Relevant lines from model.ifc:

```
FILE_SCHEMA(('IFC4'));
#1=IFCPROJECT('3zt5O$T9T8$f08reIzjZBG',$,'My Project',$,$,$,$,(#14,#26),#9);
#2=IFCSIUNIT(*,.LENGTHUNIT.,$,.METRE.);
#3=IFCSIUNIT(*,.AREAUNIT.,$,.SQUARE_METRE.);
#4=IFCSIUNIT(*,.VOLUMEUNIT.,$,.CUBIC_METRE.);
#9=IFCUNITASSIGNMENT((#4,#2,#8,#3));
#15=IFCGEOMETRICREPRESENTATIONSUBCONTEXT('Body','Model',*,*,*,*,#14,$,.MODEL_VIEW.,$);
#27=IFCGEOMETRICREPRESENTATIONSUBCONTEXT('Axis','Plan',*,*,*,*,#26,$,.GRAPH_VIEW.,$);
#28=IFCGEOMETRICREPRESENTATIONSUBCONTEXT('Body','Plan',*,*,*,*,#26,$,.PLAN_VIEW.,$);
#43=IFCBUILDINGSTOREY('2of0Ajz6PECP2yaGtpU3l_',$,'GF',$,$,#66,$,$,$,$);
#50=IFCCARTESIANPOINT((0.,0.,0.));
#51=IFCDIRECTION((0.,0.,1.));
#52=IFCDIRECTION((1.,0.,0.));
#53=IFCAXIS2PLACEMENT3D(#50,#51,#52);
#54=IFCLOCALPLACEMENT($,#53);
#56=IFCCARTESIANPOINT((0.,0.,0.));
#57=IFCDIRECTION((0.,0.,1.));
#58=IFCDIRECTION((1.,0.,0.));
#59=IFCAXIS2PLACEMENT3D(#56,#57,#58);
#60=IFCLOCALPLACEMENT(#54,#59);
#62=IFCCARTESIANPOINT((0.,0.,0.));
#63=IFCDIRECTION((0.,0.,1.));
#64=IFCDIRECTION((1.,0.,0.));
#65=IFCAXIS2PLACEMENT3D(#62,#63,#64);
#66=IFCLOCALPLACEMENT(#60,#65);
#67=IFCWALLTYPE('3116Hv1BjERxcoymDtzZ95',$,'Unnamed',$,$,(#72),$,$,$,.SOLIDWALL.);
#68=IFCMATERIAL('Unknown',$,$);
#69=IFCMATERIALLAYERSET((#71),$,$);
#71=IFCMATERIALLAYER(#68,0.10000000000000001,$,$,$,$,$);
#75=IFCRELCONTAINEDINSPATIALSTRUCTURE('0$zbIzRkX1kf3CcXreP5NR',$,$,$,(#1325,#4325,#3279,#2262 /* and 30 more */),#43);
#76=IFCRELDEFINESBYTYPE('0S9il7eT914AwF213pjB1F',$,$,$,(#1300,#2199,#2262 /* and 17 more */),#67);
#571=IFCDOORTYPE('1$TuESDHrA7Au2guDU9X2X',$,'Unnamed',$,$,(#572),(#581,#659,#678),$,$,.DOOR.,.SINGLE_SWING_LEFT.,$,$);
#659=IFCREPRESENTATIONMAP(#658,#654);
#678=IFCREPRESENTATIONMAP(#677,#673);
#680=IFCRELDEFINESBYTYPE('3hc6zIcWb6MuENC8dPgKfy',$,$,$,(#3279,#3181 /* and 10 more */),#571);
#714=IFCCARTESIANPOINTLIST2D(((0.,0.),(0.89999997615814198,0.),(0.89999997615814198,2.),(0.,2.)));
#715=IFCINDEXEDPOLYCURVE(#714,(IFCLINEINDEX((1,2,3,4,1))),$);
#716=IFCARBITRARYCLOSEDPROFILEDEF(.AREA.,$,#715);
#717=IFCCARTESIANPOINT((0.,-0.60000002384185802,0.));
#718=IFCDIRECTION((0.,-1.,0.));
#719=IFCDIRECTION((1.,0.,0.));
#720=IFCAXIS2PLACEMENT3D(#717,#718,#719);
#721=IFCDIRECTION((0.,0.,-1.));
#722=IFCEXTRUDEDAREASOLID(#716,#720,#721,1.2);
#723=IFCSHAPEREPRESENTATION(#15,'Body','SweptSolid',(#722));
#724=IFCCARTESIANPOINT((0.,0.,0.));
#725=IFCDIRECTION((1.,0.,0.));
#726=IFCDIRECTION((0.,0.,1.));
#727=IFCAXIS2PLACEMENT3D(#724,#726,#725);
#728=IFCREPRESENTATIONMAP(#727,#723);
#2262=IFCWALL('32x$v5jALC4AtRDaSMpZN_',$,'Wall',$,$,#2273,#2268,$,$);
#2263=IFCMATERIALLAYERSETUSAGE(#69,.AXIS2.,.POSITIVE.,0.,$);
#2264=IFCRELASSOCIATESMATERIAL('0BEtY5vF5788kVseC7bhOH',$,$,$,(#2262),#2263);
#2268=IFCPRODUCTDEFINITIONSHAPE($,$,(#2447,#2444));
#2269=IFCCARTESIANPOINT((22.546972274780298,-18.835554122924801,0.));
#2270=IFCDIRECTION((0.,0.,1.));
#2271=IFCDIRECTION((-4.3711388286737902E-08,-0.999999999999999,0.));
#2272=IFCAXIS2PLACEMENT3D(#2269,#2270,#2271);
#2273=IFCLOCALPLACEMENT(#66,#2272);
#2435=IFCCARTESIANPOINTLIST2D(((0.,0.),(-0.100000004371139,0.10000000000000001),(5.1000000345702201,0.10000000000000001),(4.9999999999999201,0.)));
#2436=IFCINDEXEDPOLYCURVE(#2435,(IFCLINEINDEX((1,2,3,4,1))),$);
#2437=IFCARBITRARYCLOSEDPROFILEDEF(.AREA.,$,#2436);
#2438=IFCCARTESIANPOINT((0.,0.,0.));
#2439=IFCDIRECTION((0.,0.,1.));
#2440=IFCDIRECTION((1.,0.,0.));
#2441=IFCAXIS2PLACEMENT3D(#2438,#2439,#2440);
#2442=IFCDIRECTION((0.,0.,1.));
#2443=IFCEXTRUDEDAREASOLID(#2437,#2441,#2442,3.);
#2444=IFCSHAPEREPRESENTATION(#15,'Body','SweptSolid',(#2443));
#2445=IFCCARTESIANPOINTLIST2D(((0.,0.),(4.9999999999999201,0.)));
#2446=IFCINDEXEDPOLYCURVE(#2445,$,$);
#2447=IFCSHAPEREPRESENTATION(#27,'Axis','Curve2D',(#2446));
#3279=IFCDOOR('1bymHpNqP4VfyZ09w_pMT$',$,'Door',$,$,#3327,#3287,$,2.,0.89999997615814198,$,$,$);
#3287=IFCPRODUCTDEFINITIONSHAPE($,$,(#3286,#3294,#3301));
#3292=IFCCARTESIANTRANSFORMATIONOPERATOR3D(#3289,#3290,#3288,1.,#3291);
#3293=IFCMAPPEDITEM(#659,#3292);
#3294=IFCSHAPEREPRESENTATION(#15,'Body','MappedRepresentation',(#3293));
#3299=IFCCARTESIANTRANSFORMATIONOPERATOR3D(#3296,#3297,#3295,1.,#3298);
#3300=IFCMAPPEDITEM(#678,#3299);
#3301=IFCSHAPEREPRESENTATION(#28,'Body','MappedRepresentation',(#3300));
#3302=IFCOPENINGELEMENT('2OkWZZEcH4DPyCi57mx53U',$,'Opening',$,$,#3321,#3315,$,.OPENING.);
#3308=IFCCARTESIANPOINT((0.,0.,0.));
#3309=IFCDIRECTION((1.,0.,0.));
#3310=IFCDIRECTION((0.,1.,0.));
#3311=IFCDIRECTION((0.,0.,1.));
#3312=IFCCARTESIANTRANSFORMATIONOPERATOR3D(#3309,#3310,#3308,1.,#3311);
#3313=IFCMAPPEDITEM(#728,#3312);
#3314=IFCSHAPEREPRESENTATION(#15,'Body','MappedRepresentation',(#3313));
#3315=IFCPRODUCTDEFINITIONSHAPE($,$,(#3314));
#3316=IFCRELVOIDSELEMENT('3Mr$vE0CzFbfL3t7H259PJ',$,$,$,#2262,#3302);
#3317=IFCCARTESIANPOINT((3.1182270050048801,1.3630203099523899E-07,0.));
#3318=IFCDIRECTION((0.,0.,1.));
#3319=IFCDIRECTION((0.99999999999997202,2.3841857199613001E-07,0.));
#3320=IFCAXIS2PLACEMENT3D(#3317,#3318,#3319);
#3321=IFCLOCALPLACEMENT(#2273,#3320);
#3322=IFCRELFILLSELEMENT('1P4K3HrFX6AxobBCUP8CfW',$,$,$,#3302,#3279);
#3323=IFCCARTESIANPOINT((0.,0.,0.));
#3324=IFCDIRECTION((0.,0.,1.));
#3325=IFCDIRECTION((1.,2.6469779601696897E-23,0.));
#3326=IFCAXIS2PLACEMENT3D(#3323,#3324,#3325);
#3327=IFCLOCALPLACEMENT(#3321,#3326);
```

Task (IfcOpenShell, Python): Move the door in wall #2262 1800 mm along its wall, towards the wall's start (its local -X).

```python
import ifcopenshell
import ifcopenshell.api.geometry
import ifcopenshell.util.placement
import ifcopenshell.util.unit

model = ifcopenshell.open("model.ifc")
unit_scale = ifcopenshell.util.unit.calculate_unit_scale(model)

door = model.by_guid("1bymHpNqP4VfyZ09w_pMT$")
opening = door.FillsVoids[0].RelatingOpeningElement
wall = opening.VoidsElements[0].RelatingBuildingElement

wall_matrix = ifcopenshell.util.placement.get_local_placement(wall.ObjectPlacement)
shift = wall_matrix[:3, 0] * -1.8 / unit_scale
before = ifcopenshell.util.placement.get_local_placement(door.ObjectPlacement)[:3, 3].copy()

# The door is placed relative to its opening, so it follows when the opening moves.
matrix = ifcopenshell.util.placement.get_local_placement(opening.ObjectPlacement)
matrix[:3, 3] += shift
ifcopenshell.api.geometry.edit_object_placement(
    model, product=opening, matrix=matrix, is_si=False, should_transform_children=True
)

after = ifcopenshell.util.placement.get_local_placement(door.ObjectPlacement)[:3, 3]
print("door moved by", (after - before).round(3) + 0.0)

model.write("model_v2.ifc")
```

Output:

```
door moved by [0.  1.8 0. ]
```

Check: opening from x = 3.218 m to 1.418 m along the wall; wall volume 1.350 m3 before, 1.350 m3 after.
